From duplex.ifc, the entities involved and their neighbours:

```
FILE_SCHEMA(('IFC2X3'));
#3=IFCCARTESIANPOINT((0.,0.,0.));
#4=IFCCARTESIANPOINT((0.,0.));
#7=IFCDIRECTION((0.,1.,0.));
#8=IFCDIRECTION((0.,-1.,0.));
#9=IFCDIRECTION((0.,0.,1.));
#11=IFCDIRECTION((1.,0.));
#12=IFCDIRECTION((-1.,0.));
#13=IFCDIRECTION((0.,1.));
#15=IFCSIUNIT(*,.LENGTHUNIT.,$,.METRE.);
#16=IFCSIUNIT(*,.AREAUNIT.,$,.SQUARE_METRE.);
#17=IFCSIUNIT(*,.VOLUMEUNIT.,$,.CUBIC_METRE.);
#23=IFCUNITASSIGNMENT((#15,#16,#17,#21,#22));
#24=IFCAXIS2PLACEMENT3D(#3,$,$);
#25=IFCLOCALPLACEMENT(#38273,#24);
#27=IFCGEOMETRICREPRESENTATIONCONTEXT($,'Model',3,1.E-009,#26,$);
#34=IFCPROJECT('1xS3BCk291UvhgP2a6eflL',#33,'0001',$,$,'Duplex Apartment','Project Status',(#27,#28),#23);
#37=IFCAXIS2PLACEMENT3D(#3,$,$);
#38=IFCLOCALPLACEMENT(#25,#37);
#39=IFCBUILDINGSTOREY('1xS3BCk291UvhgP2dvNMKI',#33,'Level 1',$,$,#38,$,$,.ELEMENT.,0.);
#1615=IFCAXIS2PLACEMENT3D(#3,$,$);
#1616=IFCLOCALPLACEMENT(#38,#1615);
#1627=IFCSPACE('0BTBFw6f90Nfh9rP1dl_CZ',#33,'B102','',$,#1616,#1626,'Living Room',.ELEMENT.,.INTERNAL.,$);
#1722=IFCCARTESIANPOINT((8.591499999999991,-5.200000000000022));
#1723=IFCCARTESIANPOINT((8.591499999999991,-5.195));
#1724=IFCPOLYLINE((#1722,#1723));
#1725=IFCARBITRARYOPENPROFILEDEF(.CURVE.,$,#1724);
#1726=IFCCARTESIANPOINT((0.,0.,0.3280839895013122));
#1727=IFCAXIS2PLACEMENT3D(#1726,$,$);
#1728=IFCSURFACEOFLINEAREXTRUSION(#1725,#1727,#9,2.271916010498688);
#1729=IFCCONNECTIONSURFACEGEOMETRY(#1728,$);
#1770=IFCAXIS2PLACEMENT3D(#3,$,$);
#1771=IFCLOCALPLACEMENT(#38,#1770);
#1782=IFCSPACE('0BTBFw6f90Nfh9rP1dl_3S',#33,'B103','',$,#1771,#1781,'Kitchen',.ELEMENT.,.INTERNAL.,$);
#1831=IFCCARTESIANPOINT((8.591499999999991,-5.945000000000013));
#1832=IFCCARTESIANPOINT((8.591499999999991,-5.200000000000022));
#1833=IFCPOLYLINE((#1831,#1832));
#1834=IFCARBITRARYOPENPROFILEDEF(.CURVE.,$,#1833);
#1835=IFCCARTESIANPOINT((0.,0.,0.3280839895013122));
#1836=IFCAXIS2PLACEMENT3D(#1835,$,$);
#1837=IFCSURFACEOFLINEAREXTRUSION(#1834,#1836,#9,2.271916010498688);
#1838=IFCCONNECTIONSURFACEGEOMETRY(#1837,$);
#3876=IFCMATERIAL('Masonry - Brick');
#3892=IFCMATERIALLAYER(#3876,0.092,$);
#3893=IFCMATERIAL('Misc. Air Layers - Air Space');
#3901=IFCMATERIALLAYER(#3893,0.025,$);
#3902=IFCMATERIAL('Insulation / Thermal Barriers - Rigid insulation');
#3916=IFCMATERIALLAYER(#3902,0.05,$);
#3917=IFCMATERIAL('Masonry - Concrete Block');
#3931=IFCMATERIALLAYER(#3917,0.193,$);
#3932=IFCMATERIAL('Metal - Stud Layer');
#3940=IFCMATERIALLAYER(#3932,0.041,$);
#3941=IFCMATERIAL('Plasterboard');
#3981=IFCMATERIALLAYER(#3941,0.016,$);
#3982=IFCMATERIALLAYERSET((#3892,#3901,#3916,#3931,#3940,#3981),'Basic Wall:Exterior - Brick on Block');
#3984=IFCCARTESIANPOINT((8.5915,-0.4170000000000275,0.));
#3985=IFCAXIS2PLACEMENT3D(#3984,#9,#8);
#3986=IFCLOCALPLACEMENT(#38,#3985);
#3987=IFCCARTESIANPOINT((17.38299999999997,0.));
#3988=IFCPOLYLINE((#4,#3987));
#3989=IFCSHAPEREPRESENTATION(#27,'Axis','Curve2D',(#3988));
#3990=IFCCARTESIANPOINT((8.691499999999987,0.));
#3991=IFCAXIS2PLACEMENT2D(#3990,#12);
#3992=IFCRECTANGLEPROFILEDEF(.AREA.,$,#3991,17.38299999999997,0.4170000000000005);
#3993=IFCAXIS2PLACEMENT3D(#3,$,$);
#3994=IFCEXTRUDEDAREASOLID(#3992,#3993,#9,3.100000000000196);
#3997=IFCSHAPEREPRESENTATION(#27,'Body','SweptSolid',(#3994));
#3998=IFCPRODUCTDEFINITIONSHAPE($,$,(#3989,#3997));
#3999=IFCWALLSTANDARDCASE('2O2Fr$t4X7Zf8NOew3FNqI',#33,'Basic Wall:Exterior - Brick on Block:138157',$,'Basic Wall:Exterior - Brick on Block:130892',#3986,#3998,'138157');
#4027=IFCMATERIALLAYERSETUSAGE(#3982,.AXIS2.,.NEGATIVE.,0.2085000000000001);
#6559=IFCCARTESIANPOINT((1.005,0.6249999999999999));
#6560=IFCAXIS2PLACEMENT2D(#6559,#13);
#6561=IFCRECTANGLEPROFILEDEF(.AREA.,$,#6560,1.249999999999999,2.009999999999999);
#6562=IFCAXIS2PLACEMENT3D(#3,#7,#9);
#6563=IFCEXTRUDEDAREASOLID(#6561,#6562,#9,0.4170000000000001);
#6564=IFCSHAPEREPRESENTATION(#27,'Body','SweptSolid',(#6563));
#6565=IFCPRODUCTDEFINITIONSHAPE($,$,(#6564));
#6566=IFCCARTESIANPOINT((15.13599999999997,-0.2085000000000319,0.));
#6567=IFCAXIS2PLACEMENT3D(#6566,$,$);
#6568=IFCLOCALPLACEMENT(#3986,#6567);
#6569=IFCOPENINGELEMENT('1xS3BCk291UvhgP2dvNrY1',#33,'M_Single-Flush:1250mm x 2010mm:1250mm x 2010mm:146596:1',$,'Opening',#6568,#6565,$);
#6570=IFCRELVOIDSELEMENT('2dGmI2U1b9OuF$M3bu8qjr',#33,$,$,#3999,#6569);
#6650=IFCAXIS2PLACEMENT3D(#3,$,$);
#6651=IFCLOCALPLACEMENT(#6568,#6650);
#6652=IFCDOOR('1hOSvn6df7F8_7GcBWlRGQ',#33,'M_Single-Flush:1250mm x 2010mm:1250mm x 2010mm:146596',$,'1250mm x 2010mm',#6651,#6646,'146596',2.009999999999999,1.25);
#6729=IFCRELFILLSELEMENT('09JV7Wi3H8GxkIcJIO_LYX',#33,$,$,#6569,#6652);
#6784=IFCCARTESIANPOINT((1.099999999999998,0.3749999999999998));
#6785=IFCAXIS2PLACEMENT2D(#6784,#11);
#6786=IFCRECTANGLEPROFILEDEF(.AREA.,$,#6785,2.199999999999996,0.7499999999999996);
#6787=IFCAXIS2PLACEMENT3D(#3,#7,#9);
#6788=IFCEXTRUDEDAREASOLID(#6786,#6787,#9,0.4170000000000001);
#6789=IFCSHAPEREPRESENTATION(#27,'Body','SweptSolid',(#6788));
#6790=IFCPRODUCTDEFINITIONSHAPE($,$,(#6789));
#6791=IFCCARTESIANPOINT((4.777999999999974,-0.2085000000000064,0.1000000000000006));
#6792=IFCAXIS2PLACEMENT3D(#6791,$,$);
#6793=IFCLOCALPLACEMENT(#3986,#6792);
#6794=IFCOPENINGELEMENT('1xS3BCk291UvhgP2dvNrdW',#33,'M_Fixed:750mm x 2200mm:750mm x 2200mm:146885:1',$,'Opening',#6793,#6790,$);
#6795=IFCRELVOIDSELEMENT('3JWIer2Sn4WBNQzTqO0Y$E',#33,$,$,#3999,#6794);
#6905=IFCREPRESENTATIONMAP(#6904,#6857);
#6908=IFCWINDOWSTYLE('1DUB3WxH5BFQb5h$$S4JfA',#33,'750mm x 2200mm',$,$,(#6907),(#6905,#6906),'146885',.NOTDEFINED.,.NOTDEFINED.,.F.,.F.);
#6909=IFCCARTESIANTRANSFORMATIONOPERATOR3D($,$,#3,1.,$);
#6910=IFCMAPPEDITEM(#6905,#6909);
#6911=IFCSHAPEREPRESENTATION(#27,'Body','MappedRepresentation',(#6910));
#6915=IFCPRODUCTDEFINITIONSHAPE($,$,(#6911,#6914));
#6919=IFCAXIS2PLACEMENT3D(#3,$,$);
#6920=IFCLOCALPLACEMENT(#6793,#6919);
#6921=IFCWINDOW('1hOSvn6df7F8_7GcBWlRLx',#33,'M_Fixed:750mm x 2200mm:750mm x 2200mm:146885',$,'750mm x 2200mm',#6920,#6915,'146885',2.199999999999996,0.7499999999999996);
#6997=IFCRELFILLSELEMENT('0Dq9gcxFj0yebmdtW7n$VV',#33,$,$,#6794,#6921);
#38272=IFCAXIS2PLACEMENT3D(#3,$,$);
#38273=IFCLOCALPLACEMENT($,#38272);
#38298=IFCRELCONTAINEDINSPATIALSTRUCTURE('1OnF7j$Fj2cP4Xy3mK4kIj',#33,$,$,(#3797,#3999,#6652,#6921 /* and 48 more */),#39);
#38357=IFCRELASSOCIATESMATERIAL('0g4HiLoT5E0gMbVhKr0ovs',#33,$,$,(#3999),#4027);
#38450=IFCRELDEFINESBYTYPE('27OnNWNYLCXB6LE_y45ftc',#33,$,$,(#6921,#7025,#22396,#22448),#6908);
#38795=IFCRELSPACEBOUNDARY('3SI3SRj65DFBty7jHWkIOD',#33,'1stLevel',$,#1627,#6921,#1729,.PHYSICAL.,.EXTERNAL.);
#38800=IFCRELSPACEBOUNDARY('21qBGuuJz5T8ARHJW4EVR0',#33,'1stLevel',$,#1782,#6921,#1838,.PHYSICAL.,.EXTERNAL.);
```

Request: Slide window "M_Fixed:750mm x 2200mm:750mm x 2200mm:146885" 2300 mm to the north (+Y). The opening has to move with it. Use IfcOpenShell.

```python
import numpy as np
import ifcopenshell
import ifcopenshell.api.geometry
import ifcopenshell.util.placement

model = ifcopenshell.open("duplex.ifc")

window = model.by_guid("1hOSvn6df7F8_7GcBWlRLx")
opening = window.FillsVoids[0].RelatingOpeningElement
wall = opening.VoidsElements[0].RelatingBuildingElement

wall_matrix = ifcopenshell.util.placement.get_local_placement(wall.ObjectPlacement)
shift = wall_matrix[:3, 0] * -2.3
before = ifcopenshell.util.placement.get_local_placement(window.ObjectPlacement)[:3, 3].copy()

# The window is placed relative to its opening, so it follows when the opening moves.
matrix = ifcopenshell.util.placement.get_local_placement(opening.ObjectPlacement)
matrix[:3, 3] += shift
ifcopenshell.api.geometry.edit_object_placement(
    model, product=opening, matrix=matrix, is_si=False, should_transform_children=True
)

# Space boundary surfaces are stored in each space's coordinates; move them too.
for rel in window.ProvidesBoundaries:
    if not rel.ConnectionGeometry:
        continue
    surface = rel.ConnectionGeometry.SurfaceOnRelatingElement
    space_matrix = ifcopenshell.util.placement.get_local_placement(rel.RelatingSpace.ObjectPlacement)
    point = np.array(surface.Position.Location.Coordinates) + space_matrix[:3, :3].T @ shift
    surface.Position = model.createIfcAxis2Placement3D(
        model.createIfcCartesianPoint(point.tolist()), surface.Position.Axis, surface.Position.RefDirection
    )

after = ifcopenshell.util.placement.get_local_placement(window.ObjectPlacement)[:3, 3]
print("window moved by", (after - before).round(3) + 0.0)

model.write("duplex-out.ifc")
```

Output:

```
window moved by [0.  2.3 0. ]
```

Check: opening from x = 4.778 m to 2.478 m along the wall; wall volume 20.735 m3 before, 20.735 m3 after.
